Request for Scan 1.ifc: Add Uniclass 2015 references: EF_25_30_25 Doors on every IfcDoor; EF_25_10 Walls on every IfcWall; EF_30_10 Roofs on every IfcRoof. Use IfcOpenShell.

First a look at what the model holds.

```python
import ifcopenshell

model = ifcopenshell.open("Scan 1.ifc")
print(model.schema)
print("classifications:", [c.Name for c in model.by_type("IfcClassification")])
for ifc_class in ("IfcDoor", "IfcRoof", "IfcStair", "IfcWall", "IfcWindow"):
    print(ifc_class, len(model.by_type(ifc_class)))
```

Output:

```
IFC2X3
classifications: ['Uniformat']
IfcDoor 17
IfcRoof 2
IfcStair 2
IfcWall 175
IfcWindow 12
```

```python
import ifcopenshell
import ifcopenshell.api.classification

model = ifcopenshell.open("Scan 1.ifc")

# IFC2X3 requires Source and Edition and has no link from the project to the system.
system = model.create_entity("IfcClassification", Source="NBS", Edition="2015", Name="Uniclass 2015")

codes = {
    "IfcDoor": ("EF_25_30_25", "Doors"),
    "IfcWall": ("EF_25_10", "Walls"),
    "IfcRoof": ("EF_30_10", "Roofs"),
}
for ifc_class, (code, name) in codes.items():
    products = model.by_type(ifc_class)
    ifcopenshell.api.classification.add_reference(
        model, products=products, classification=system, identification=code, name=name
    )
    print(code, len(products))

model.write("Scan 1-out.ifc")
```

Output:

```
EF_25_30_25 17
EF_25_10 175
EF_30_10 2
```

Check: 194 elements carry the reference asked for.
